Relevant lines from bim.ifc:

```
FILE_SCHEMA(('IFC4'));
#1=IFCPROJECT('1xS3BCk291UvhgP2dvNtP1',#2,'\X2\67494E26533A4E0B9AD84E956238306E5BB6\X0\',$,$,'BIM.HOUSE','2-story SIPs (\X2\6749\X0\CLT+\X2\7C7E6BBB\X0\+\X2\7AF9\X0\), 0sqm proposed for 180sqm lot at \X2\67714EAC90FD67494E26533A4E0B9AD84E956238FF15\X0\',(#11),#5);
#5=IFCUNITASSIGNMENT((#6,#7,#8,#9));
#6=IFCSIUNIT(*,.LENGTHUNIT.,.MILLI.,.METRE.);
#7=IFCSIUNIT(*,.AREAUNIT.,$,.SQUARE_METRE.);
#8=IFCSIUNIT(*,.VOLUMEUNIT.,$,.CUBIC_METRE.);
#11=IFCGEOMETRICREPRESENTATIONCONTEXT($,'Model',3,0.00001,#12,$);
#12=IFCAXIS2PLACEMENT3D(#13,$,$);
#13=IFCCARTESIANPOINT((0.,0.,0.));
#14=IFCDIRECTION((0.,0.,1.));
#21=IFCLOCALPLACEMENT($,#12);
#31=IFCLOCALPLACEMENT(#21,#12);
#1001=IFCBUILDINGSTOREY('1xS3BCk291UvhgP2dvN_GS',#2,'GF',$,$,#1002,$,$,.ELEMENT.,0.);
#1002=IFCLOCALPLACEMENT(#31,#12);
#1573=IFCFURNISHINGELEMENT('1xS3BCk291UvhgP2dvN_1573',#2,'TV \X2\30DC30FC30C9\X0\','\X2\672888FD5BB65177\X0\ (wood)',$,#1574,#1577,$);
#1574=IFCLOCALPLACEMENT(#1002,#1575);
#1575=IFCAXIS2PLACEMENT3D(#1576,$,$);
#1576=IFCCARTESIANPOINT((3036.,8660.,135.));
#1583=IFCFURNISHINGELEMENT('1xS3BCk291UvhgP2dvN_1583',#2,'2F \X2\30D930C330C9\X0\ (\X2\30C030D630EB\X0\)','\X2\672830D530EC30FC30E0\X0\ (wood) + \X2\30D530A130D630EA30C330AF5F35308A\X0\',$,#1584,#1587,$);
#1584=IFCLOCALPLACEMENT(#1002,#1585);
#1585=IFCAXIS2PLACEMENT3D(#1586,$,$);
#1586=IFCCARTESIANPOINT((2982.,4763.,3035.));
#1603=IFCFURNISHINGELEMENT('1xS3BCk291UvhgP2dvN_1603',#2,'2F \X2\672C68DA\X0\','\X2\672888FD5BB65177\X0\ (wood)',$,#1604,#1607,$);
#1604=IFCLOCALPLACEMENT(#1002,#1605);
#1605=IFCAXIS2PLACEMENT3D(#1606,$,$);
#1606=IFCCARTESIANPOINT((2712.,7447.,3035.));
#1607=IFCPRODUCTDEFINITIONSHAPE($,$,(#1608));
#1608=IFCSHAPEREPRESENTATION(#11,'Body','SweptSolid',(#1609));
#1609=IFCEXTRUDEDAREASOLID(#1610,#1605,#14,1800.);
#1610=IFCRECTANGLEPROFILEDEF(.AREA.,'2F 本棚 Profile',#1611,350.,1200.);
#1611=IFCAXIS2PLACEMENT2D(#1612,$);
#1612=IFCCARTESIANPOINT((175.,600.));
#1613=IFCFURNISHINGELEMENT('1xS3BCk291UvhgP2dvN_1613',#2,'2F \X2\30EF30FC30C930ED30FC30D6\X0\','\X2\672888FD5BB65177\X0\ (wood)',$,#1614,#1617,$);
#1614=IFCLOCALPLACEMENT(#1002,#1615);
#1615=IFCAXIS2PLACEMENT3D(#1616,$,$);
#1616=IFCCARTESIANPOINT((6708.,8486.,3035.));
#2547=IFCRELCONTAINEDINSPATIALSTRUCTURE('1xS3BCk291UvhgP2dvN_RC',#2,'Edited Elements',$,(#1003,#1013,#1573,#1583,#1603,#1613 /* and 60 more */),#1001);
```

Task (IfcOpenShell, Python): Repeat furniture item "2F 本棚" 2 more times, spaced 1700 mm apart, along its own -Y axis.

```python
import ifcopenshell
import ifcopenshell.api.geometry
import ifcopenshell.api.root
import ifcopenshell.util.element
import ifcopenshell.util.placement

model = ifcopenshell.open("bim.ifc")


def reuse_history(source, copy):
    """copy_class also copies each property set's owner history, people and application; keep the originals."""
    for rel in copy.IsDefinedBy:
        if rel.is_a("IfcRelDefinesByProperties") and (history := rel.RelatingPropertyDefinition.OwnerHistory):
            rel.RelatingPropertyDefinition.OwnerHistory = source.OwnerHistory
            ifcopenshell.util.element.remove_deep2(model, history)


source = model.by_id(1603)
base = ifcopenshell.util.placement.get_local_placement(source.ObjectPlacement)
step = -base[:3, 1] * 1700.0

for i in range(1, 3):
    copy = ifcopenshell.api.root.copy_class(model, product=source)
    copy.Representation = ifcopenshell.util.element.copy_deep(
        model, source.Representation, exclude=["IfcGeometricRepresentationContext", "IfcRepresentationMap"]
    )
    reuse_history(source, copy)
    matrix = base.copy()
    matrix[:3, 3] += i * step
    print("added at", matrix[:3, 3].round(3) + 0.0)
    ifcopenshell.api.geometry.edit_object_placement(model, product=copy, matrix=matrix, is_si=False)

model.write("bim_v2.ifc")
```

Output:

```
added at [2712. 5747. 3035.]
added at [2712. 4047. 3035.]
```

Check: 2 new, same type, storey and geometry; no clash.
